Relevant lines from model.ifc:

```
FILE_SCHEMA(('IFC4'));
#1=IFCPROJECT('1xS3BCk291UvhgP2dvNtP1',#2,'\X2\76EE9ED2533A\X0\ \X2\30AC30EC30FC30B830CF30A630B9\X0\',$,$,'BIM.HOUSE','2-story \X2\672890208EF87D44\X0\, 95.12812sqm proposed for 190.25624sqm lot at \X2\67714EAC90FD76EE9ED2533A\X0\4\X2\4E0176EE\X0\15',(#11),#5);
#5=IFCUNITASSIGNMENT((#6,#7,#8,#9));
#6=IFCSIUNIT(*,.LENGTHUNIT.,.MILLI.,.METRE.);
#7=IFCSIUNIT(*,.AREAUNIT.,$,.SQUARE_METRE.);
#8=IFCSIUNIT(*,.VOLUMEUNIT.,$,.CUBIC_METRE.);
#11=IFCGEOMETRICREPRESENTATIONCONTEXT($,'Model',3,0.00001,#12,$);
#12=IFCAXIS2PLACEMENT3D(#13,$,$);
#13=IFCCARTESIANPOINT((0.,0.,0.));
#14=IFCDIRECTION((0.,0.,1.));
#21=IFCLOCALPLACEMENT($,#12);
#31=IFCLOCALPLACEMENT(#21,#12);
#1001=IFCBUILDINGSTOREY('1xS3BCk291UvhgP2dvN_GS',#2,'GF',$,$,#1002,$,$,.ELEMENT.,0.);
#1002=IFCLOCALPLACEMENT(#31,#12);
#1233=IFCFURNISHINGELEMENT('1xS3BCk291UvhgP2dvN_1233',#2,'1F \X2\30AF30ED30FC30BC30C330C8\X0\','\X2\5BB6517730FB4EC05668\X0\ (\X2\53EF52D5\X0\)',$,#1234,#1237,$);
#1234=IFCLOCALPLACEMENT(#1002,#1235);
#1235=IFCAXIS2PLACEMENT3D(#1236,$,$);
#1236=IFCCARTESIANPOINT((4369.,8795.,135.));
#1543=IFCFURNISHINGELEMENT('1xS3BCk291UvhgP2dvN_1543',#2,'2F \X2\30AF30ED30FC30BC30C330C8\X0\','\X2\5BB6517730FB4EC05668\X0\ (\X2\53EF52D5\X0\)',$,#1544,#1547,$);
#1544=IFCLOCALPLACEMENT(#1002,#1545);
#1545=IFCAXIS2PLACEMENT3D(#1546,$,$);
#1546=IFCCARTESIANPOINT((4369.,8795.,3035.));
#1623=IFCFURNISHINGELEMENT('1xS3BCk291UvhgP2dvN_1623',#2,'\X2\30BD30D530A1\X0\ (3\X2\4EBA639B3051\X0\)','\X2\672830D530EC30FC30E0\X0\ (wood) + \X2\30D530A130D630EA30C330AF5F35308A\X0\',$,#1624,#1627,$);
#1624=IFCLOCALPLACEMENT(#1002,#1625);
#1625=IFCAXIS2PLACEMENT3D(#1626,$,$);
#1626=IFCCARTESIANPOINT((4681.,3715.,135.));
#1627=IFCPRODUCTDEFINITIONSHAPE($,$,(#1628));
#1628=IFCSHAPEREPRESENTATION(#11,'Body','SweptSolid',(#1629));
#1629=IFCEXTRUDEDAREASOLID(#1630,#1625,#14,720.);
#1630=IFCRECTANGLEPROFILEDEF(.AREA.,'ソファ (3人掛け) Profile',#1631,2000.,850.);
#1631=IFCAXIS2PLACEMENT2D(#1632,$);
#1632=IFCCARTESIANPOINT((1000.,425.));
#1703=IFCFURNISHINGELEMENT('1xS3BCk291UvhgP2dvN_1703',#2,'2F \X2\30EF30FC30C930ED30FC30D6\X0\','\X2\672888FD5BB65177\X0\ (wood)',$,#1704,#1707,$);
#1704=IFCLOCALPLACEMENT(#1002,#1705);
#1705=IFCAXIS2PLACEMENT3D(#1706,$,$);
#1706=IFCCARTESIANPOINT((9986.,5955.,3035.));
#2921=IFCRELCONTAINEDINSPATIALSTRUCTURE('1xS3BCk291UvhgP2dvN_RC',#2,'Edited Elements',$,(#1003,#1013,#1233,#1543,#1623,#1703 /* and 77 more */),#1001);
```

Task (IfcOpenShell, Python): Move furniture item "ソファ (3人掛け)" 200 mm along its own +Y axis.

```python
import ifcopenshell
import ifcopenshell.api.geometry
import ifcopenshell.util.placement
import ifcopenshell.util.unit

model = ifcopenshell.open("model.ifc")
unit_scale = ifcopenshell.util.unit.calculate_unit_scale(model)

item = model.by_guid("1xS3BCk291UvhgP2dvN_1623")
matrix = ifcopenshell.util.placement.get_local_placement(item.ObjectPlacement)
matrix[:3, 3] += matrix[:3, 1] * 0.2 / unit_scale
ifcopenshell.api.geometry.edit_object_placement(model, product=item, matrix=matrix, is_si=False)

print(ifcopenshell.util.placement.get_local_placement(item.ObjectPlacement).round(3) + 0.0)

model.write("model_v2.ifc")
```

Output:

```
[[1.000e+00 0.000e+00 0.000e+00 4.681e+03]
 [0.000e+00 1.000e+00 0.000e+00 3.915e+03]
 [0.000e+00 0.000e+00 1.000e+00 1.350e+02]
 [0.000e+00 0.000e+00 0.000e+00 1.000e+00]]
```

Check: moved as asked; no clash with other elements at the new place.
